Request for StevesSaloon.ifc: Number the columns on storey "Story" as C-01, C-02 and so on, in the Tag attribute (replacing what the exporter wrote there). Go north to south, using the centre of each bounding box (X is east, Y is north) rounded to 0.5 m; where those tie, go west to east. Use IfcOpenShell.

First a look at what the model holds.

```python
import ifcopenshell
import ifcopenshell.util.element
import ifcopenshell.util.placement

model = ifcopenshell.open("StevesSaloon.ifc")
print(model.schema)
storey = next(s for s in model.by_type("IfcBuildingStorey") if s.Name == "Story")
columns = [e for e in ifcopenshell.util.element.get_decomposition(storey) if e.is_a("IfcColumn")]
for e in sorted(columns, key=lambda e: e.id()):
    origin = ifcopenshell.util.placement.get_local_placement(e.ObjectPlacement)[:3, 3]
    print(e.id(), e.Tag, e.Name, origin.round(2) + 0.0, sep=" | ")
```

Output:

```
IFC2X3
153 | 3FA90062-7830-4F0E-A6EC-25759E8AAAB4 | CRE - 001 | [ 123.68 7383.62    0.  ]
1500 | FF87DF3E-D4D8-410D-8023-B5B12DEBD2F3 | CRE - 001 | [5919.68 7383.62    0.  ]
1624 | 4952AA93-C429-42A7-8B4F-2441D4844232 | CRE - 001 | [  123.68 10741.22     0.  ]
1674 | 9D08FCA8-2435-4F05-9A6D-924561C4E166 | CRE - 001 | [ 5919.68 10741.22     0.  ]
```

```python
import ifcopenshell
import ifcopenshell.geom
import ifcopenshell.util.element
import ifcopenshell.util.shape

model = ifcopenshell.open("StevesSaloon.ifc")
settings = ifcopenshell.geom.settings()
settings.set("use-world-coords", True)


def centre(element):
    shape = ifcopenshell.geom.create_shape(settings, element)
    return ifcopenshell.util.shape.get_bbox_centroid(shape.geometry)


storey = next(s for s in model.by_type("IfcBuildingStorey") if s.Name == "Story")
columns = [e for e in ifcopenshell.util.element.get_decomposition(storey) if e.is_a("IfcColumn")]

# Insertion points can sit at a corner or the storey origin, so sort by the geometry (in metres).
centres = {e: centre(e) for e in columns}
columns.sort(key=lambda e: (-round(centres[e][1] / 0.5), centres[e][0]))

for i, e in enumerate(columns, start=1):
    number = f"C-{i:02d}"
    e.Tag = number
    print(e.id(), number)

model.write("StevesSaloon_updated.ifc")
```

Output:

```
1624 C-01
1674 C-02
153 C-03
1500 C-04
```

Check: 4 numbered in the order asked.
